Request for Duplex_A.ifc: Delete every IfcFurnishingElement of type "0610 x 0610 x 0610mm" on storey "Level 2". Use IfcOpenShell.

First a look at what the model holds.

```python
import ifcopenshell
import ifcopenshell.util.element

model = ifcopenshell.open("Duplex_A.ifc")
print(model.schema)
storey = next(s for s in model.by_type("IfcBuildingStorey") if s.Name == "Level 2")
furniture = [e for e in ifcopenshell.util.element.get_decomposition(storey) if e.is_a("IfcFurnishingElement")]
seen = {}
for e in furniture:
    element_type = ifcopenshell.util.element.get_type(e)
    name = element_type.Name if element_type not in (None, e) else None
    seen[name] = seen.get(name, 0) + 1
for name, count in sorted(seen.items(), key=str):
    print(count, "x", name)
```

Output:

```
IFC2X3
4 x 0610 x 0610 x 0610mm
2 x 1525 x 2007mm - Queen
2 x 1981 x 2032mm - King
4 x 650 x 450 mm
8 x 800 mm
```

```python
import ifcopenshell
import ifcopenshell.api.root
import ifcopenshell.util.element

model = ifcopenshell.open("Duplex_A.ifc")

storey = next(s for s in model.by_type("IfcBuildingStorey") if s.Name == "Level 2")
furniture = [e for e in ifcopenshell.util.element.get_decomposition(storey) if e.is_a("IfcFurnishingElement")]
targets = [e for e in furniture if (t := ifcopenshell.util.element.get_type(e)) not in (None, e) and t.Name == "0610 x 0610 x 0610mm"]

for e in targets:
    ifcopenshell.api.root.remove_product(model, product=e)
print(len(targets), "removed")

model.write("Duplex_A_v2.ifc")
```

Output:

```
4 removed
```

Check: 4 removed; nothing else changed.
